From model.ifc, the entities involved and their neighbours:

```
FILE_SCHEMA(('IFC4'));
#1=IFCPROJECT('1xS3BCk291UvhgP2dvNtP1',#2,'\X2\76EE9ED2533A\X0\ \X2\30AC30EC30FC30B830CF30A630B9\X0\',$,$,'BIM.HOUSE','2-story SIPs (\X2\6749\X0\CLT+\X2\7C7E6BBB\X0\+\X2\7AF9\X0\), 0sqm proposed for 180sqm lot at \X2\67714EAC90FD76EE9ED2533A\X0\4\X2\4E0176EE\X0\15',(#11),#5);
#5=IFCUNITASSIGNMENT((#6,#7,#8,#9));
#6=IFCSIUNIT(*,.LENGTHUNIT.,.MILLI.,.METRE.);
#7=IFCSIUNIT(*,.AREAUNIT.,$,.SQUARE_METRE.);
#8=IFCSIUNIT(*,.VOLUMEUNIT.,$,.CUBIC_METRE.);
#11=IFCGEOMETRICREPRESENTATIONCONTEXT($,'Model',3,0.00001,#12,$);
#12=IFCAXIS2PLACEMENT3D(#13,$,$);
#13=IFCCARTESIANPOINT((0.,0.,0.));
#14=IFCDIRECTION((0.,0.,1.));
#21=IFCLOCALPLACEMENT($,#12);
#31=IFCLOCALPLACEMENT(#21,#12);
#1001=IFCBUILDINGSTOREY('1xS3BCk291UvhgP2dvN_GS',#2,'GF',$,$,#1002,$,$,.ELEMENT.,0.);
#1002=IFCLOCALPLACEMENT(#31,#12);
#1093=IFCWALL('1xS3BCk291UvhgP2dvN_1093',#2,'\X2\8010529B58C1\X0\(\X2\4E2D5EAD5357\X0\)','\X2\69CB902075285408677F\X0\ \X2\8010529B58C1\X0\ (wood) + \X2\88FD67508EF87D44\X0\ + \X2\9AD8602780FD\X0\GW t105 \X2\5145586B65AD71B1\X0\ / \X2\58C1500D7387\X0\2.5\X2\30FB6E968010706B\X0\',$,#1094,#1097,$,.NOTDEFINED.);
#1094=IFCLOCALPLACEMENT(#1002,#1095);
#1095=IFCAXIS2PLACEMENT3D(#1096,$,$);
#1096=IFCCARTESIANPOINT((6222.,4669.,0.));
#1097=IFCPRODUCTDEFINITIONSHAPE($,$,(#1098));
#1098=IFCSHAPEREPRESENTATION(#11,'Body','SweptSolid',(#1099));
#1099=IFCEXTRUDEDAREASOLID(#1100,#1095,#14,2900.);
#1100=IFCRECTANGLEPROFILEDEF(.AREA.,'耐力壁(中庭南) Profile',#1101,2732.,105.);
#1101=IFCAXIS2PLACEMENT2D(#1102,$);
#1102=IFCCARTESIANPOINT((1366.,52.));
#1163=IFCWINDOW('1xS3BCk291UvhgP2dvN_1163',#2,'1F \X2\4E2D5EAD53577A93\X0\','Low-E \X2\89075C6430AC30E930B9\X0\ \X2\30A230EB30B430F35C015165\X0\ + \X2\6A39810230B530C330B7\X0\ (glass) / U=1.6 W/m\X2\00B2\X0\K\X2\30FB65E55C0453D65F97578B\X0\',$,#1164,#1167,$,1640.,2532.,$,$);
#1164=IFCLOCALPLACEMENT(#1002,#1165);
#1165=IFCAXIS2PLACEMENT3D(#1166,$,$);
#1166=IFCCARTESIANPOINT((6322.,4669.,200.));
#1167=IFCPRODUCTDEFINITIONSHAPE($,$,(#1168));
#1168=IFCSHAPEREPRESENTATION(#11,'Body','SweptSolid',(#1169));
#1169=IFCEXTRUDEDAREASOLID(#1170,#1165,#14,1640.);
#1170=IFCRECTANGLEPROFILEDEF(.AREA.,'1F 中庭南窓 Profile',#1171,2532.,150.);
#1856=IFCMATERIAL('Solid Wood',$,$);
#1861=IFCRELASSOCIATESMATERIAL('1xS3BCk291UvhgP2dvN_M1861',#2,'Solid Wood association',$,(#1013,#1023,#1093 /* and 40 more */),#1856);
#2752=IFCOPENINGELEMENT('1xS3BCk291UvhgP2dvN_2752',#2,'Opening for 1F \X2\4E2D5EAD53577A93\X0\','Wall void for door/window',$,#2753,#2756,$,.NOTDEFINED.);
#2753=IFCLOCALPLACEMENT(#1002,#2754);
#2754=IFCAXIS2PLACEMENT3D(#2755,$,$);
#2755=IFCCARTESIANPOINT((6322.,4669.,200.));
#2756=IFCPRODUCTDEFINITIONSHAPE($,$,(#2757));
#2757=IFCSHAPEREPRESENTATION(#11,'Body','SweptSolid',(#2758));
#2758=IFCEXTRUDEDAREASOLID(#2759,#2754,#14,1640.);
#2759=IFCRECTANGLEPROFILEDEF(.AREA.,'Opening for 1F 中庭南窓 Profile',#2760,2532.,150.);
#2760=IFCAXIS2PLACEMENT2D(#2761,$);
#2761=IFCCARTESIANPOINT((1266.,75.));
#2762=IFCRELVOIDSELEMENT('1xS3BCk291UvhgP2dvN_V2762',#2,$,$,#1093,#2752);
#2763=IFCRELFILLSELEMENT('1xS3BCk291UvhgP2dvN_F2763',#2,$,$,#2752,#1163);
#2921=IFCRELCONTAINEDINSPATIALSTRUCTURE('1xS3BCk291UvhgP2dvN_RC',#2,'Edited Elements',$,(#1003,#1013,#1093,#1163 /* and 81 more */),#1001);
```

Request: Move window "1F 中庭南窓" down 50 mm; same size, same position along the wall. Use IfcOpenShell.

```python
import numpy as np
import ifcopenshell
import ifcopenshell.api.geometry
import ifcopenshell.util.placement
import ifcopenshell.util.unit

model = ifcopenshell.open("model.ifc")
unit_scale = ifcopenshell.util.unit.calculate_unit_scale(model)

window = model.by_id(1163)
opening = window.FillsVoids[0].RelatingOpeningElement
dz = -0.05 / unit_scale

shift = np.array([0.0, 0.0, dz])
# The window is not placed relative to its opening, so move both.
for product in (opening, window):
    matrix = ifcopenshell.util.placement.get_local_placement(product.ObjectPlacement)
    matrix[:3, 3] += shift
    ifcopenshell.api.geometry.edit_object_placement(model, product=product, matrix=matrix, is_si=False)

print(f"moved by {dz * unit_scale:+.3f} m")

model.write("model_updated.ifc")
```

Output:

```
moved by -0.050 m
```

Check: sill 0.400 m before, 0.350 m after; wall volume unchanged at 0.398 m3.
